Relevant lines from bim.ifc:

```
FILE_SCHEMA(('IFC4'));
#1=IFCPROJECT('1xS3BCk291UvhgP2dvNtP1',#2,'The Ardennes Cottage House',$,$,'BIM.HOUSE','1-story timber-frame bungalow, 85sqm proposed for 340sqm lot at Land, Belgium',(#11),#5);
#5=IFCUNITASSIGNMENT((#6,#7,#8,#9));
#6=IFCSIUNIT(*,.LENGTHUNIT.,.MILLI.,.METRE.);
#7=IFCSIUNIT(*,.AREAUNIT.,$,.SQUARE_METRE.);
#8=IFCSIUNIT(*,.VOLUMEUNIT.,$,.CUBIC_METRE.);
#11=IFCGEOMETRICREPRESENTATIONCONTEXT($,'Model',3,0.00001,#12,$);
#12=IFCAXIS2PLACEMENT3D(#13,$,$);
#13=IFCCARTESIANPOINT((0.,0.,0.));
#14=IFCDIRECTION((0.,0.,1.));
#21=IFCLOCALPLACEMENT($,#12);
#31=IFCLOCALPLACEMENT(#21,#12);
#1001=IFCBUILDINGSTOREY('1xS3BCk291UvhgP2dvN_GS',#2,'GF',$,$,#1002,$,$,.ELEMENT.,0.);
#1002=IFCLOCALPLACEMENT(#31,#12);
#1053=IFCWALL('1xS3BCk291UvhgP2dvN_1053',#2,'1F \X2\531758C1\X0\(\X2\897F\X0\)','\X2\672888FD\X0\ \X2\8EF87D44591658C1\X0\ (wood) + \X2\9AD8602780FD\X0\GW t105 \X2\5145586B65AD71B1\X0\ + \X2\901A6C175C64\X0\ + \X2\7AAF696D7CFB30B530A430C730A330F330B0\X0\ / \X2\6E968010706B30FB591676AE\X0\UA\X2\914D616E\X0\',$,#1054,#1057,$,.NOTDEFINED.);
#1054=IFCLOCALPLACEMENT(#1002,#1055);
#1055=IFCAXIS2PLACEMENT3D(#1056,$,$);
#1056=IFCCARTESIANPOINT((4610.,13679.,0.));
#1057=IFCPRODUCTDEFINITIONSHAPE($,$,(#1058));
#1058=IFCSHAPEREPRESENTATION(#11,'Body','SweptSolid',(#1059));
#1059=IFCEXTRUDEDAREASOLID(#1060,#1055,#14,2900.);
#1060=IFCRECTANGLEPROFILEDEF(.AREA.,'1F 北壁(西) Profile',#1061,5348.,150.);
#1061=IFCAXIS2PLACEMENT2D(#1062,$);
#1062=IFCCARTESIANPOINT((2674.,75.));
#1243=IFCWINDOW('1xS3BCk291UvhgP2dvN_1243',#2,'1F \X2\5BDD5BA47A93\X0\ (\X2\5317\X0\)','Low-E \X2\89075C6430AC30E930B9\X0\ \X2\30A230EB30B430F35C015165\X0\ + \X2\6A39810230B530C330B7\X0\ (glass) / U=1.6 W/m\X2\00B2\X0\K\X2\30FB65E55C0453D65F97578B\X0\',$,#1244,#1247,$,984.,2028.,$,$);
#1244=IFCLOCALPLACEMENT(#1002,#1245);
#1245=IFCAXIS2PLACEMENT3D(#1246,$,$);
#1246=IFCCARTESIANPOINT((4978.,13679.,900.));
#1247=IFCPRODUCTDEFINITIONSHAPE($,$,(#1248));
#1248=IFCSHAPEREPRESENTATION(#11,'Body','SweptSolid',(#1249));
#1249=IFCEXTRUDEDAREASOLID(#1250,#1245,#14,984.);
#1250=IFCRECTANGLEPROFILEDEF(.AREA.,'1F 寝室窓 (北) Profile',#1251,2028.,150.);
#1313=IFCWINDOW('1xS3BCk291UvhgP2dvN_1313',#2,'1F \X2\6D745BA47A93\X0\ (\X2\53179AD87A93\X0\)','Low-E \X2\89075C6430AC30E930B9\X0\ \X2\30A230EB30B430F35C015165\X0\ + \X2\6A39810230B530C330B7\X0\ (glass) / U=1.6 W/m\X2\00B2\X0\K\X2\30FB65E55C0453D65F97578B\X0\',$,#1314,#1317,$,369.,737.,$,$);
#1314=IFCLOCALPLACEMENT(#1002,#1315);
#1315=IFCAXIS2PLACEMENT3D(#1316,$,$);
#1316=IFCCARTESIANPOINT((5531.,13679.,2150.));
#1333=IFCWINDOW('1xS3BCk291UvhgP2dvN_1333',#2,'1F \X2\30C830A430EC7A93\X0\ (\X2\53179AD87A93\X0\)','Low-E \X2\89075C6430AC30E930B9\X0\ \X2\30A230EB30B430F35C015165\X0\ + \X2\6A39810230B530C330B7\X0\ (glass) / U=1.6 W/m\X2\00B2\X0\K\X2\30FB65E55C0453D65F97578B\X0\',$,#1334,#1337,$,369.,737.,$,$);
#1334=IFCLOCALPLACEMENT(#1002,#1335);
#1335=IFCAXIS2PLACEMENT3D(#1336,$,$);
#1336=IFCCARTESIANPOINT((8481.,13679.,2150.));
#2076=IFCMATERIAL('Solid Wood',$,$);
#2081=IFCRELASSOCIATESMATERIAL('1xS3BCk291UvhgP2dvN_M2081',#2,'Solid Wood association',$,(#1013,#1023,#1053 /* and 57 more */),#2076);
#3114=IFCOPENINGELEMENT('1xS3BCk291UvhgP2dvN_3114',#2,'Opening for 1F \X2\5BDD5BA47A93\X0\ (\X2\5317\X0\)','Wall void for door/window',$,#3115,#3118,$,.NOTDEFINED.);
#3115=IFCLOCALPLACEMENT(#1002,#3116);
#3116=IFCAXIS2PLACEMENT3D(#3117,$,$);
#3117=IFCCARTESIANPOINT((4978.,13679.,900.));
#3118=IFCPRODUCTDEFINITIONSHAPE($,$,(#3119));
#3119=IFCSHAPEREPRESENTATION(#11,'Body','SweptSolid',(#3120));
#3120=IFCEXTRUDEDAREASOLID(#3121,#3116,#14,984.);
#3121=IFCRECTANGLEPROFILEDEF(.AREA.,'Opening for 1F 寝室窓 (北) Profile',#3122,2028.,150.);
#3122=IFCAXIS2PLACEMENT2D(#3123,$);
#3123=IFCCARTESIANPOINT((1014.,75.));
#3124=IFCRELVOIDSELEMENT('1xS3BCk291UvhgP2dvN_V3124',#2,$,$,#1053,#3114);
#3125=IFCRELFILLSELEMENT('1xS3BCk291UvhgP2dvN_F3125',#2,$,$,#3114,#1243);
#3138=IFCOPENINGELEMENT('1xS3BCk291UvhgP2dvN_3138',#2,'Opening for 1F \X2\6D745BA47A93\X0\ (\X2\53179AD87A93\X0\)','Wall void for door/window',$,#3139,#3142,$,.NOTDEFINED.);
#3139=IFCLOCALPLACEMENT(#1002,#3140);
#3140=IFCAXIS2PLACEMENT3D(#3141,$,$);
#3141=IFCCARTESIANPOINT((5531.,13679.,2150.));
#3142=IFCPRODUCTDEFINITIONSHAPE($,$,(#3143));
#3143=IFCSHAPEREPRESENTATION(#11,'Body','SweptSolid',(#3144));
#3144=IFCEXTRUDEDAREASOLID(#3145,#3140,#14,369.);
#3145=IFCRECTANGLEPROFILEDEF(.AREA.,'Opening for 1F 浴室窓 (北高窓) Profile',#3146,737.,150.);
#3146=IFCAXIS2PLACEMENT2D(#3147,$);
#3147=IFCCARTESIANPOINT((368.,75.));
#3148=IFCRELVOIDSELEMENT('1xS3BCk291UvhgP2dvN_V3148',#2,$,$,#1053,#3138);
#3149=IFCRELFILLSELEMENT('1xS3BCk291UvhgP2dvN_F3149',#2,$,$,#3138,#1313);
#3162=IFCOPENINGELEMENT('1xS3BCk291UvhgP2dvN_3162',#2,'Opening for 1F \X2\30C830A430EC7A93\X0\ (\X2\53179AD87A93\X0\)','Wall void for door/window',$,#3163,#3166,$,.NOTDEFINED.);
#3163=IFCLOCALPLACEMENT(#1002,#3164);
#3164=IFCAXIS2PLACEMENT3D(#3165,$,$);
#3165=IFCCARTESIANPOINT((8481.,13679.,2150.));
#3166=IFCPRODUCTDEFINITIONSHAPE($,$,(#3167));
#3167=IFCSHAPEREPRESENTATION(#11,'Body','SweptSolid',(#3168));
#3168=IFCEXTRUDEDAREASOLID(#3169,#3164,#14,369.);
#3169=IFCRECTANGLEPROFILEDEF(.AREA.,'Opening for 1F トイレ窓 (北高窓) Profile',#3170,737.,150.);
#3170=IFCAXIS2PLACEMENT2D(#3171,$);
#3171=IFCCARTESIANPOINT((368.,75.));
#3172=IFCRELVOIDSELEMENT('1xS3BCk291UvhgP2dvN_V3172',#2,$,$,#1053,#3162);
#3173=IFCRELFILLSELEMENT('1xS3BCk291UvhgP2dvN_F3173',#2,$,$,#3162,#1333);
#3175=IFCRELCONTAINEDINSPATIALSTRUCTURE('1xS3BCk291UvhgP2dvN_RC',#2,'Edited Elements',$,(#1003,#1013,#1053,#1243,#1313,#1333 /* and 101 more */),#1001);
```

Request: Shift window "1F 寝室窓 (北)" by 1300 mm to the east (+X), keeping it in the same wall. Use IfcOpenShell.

```python
import ifcopenshell
import ifcopenshell.api.geometry
import ifcopenshell.util.placement
import ifcopenshell.util.unit

model = ifcopenshell.open("bim.ifc")
unit_scale = ifcopenshell.util.unit.calculate_unit_scale(model)

window = model.by_guid("1xS3BCk291UvhgP2dvN_1243")
opening = window.FillsVoids[0].RelatingOpeningElement
wall = opening.VoidsElements[0].RelatingBuildingElement

wall_matrix = ifcopenshell.util.placement.get_local_placement(wall.ObjectPlacement)
shift = wall_matrix[:3, 0] * 1.3 / unit_scale
before = ifcopenshell.util.placement.get_local_placement(window.ObjectPlacement)[:3, 3].copy()

# The window is not placed relative to its opening, so move both.
for product in (opening, window):
    matrix = ifcopenshell.util.placement.get_local_placement(product.ObjectPlacement)
    matrix[:3, 3] += shift
    ifcopenshell.api.geometry.edit_object_placement(model, product=product, matrix=matrix, is_si=False)

after = ifcopenshell.util.placement.get_local_placement(window.ObjectPlacement)[:3, 3]
print("window moved by", (after - before).round(3) + 0.0)

model.write("bim_updated.ifc")
```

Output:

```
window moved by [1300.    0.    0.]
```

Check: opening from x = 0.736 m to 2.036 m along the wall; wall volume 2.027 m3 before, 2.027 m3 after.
